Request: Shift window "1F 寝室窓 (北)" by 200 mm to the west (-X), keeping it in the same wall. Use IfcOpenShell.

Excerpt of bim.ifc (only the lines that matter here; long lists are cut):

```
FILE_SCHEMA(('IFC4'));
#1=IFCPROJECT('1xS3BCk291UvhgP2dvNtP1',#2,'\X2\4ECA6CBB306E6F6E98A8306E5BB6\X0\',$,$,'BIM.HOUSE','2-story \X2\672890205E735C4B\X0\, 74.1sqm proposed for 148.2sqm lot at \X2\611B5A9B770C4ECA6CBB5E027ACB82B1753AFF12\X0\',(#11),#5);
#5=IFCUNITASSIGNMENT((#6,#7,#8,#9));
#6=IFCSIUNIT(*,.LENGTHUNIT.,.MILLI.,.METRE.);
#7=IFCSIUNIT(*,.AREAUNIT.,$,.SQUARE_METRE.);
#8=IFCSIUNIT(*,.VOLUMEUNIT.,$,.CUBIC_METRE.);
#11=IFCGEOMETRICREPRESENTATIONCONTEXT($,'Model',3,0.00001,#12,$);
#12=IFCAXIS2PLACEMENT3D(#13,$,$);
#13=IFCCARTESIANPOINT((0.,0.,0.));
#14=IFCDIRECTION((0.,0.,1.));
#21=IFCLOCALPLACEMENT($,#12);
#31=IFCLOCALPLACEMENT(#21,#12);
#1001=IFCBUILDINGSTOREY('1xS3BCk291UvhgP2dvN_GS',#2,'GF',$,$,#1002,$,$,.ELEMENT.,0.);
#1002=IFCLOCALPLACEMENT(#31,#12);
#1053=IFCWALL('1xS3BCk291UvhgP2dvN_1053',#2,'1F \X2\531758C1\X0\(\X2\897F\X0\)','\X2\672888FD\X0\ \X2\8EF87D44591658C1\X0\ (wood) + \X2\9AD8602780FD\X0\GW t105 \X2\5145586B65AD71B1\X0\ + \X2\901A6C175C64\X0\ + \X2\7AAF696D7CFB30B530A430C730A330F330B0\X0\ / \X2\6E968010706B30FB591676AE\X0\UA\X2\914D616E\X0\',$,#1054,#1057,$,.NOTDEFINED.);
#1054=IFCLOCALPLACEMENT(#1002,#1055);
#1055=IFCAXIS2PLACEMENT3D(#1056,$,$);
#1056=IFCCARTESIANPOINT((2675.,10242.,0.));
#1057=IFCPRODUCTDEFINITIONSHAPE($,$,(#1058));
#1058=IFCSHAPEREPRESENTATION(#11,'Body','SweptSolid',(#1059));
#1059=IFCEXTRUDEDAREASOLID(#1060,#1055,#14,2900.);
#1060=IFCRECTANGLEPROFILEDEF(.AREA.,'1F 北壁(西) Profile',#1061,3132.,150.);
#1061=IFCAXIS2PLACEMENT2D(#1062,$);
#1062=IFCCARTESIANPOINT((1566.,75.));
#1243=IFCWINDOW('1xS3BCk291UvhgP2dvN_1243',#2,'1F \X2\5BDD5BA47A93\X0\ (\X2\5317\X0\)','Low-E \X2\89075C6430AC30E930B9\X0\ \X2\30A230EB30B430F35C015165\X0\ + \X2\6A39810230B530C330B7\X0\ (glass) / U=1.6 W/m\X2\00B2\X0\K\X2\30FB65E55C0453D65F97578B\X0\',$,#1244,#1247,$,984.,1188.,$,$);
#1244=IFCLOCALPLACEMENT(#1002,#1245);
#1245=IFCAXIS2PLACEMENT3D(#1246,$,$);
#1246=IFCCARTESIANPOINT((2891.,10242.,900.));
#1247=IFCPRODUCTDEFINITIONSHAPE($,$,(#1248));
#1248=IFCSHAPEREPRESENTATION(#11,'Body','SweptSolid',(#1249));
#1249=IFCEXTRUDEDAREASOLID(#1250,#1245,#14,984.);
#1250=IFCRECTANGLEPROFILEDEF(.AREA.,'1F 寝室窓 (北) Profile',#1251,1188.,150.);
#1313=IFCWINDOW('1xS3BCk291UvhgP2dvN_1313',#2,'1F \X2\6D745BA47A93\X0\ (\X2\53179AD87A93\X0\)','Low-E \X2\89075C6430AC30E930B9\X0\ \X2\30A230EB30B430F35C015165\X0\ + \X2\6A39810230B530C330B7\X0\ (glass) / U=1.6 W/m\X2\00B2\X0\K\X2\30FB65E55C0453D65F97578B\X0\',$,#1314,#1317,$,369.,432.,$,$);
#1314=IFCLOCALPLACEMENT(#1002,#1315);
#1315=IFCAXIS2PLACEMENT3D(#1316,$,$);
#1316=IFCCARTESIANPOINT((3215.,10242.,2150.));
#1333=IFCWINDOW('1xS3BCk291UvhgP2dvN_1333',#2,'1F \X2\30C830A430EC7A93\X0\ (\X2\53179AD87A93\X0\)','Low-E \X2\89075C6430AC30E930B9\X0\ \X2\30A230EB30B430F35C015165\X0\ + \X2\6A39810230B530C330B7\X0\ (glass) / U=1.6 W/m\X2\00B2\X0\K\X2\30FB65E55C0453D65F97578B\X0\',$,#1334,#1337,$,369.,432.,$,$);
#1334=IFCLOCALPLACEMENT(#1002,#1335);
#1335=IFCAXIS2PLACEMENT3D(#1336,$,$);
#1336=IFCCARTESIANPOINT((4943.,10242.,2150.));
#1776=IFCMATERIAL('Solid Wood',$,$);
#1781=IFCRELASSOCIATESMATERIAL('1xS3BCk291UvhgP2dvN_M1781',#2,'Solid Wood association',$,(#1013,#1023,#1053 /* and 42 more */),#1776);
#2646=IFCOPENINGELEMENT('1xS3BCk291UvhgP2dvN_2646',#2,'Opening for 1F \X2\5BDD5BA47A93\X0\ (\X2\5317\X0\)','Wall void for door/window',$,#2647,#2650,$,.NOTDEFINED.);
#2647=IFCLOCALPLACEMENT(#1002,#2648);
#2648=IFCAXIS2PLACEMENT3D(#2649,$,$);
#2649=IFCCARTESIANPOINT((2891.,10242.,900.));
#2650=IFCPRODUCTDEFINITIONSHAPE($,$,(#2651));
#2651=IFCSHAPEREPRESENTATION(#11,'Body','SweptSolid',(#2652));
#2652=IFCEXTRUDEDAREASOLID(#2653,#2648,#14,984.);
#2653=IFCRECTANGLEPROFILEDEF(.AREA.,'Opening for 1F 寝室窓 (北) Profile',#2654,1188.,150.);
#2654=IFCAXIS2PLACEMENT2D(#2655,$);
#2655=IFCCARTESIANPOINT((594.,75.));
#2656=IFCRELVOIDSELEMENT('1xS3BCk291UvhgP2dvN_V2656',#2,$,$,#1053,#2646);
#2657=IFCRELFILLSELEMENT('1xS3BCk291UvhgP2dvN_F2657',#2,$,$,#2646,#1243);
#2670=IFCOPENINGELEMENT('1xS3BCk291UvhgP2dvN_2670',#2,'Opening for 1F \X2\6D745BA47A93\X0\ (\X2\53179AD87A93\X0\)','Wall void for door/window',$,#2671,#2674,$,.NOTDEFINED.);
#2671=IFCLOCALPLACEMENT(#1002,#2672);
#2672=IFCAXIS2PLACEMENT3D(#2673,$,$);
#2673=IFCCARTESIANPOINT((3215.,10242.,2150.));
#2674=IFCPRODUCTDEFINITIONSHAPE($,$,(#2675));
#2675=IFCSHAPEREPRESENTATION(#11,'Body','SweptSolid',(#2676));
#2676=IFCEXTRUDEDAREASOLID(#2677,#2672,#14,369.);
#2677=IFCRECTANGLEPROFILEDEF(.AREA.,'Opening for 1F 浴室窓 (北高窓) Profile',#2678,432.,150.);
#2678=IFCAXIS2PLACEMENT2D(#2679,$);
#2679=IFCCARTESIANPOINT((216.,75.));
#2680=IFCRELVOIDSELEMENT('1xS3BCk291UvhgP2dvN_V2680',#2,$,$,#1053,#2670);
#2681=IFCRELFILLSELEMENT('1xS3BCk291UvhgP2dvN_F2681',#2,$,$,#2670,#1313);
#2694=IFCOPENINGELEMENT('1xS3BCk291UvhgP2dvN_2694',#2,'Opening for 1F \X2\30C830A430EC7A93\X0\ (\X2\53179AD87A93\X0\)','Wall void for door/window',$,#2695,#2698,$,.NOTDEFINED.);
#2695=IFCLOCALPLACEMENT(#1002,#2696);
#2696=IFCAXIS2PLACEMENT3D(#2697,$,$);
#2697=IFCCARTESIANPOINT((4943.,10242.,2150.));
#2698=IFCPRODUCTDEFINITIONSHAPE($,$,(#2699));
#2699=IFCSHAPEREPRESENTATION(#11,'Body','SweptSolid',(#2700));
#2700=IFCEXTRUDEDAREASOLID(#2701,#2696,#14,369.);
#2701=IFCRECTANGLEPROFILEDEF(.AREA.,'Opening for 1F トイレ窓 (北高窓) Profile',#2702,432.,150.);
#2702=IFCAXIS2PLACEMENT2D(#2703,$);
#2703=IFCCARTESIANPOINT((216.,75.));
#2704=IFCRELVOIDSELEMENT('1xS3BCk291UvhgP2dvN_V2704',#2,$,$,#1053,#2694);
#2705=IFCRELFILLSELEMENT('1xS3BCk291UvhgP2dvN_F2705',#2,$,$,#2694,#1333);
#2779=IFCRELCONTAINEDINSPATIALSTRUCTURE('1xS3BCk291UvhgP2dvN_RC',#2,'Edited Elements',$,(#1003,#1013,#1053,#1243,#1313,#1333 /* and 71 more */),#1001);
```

```python
import ifcopenshell
import ifcopenshell.api.geometry
import ifcopenshell.util.placement
import ifcopenshell.util.unit

model = ifcopenshell.open("bim.ifc")
unit_scale = ifcopenshell.util.unit.calculate_unit_scale(model)

window = model.by_guid("1xS3BCk291UvhgP2dvN_1243")
opening = window.FillsVoids[0].RelatingOpeningElement
wall = opening.VoidsElements[0].RelatingBuildingElement

wall_matrix = ifcopenshell.util.placement.get_local_placement(wall.ObjectPlacement)
shift = wall_matrix[:3, 0] * -0.2 / unit_scale
before = ifcopenshell.util.placement.get_local_placement(window.ObjectPlacement)[:3, 3].copy()

# The window is not placed relative to its opening, so move both.
for product in (opening, window):
    matrix = ifcopenshell.util.placement.get_local_placement(product.ObjectPlacement)
    matrix[:3, 3] += shift
    ifcopenshell.api.geometry.edit_object_placement(model, product=product, matrix=matrix, is_si=False)

after = ifcopenshell.util.placement.get_local_placement(window.ObjectPlacement)[:3, 3]
print("window moved by", (after - before).round(3) + 0.0)

model.write("bim_rev.ifc")
```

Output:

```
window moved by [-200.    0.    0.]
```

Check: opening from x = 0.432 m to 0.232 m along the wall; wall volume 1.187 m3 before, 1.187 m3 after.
